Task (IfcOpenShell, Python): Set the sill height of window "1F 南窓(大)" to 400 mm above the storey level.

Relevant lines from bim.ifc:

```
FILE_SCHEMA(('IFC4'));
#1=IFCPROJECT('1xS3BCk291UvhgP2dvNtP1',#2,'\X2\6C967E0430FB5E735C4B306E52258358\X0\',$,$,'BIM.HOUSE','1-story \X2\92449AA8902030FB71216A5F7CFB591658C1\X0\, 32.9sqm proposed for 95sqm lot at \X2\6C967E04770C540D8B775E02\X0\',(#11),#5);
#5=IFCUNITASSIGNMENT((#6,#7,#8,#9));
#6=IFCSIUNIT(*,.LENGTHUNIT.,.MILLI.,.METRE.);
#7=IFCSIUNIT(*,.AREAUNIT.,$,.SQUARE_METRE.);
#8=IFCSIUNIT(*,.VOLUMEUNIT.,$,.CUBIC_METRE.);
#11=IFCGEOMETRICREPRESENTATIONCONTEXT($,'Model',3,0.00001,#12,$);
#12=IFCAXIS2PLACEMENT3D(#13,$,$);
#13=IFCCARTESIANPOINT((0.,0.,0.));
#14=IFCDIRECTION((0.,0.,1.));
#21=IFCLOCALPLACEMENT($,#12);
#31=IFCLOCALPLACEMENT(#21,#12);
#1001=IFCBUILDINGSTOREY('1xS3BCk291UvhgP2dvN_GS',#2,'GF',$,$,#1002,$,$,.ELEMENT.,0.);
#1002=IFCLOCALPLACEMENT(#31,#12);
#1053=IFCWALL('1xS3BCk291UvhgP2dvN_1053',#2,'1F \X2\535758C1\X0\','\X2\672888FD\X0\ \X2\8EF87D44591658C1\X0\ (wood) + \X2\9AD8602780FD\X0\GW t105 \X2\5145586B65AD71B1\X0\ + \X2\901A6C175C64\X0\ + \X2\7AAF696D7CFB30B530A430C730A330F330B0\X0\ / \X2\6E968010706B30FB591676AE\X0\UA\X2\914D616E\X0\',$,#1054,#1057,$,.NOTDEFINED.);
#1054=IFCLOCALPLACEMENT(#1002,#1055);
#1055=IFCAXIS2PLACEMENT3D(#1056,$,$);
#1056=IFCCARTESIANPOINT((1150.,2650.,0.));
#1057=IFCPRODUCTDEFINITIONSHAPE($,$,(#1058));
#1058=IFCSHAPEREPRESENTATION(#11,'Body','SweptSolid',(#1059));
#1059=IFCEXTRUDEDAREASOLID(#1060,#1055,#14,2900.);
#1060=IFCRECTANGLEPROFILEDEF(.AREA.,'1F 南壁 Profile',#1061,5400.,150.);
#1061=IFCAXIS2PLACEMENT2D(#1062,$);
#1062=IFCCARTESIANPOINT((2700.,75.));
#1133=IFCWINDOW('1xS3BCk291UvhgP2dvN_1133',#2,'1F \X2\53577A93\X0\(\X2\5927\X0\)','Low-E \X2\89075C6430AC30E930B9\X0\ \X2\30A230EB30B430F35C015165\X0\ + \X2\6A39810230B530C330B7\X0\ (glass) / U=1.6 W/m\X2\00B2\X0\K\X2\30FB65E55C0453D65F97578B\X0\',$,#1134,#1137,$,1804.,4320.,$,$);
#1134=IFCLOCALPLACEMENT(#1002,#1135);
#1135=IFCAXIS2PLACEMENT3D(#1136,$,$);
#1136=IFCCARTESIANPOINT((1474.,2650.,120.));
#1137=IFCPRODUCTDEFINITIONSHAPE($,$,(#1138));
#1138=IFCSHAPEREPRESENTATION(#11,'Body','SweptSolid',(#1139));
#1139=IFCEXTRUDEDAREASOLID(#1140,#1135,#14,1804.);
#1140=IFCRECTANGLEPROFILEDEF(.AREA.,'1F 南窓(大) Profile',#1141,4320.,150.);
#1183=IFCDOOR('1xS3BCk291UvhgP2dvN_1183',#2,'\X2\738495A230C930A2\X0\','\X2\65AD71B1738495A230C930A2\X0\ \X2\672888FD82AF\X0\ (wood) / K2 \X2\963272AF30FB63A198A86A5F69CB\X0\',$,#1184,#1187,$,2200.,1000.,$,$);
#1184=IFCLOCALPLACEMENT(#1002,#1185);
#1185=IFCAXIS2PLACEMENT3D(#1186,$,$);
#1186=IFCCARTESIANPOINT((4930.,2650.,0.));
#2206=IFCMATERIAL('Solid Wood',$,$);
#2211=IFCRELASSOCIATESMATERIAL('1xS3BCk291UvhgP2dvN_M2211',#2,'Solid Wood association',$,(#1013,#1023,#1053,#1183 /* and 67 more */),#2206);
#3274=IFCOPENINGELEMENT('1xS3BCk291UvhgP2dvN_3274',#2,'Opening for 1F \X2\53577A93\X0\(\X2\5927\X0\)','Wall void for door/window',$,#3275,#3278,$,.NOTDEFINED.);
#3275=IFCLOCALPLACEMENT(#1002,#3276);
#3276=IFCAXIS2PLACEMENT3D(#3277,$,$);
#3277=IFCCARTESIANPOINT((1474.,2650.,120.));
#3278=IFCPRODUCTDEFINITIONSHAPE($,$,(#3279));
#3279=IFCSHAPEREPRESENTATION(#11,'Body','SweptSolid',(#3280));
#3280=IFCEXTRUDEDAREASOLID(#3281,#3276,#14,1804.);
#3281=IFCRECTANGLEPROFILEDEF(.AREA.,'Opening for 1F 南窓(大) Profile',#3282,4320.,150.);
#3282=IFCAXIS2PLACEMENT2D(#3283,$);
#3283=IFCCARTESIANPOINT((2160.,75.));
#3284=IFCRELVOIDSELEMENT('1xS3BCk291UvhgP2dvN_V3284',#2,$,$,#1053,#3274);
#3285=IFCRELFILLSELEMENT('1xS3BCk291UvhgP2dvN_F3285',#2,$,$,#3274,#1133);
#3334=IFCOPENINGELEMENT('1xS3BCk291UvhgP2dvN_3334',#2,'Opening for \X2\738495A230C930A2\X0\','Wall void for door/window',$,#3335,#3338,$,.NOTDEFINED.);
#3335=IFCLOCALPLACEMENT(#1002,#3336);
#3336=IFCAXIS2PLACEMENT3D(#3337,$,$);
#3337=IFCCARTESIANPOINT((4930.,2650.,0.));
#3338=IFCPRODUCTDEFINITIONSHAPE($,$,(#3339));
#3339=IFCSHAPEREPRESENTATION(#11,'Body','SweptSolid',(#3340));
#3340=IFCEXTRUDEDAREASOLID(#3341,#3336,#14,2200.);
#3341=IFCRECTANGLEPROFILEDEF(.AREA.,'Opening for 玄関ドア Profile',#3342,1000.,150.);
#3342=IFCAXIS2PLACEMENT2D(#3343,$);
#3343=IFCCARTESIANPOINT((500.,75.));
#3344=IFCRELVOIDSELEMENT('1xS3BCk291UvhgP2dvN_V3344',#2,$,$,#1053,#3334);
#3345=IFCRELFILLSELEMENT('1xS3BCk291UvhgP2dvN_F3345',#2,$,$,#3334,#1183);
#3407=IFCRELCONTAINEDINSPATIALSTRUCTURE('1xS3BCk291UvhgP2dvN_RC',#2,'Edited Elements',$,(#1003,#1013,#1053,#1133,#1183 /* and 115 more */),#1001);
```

```python
import numpy as np
import ifcopenshell
import ifcopenshell.api.geometry
import ifcopenshell.geom
import ifcopenshell.util.element
import ifcopenshell.util.placement
import ifcopenshell.util.shape
import ifcopenshell.util.unit

model = ifcopenshell.open("bim.ifc")
unit_scale = ifcopenshell.util.unit.calculate_unit_scale(model)

window = model.by_guid("1xS3BCk291UvhgP2dvN_1133")
opening = window.FillsVoids[0].RelatingOpeningElement
storey = ifcopenshell.util.element.get_container(window, ifc_class="IfcBuildingStorey")
level = ifcopenshell.util.placement.get_local_placement(storey.ObjectPlacement)[2, 3]

# The opening's origin need not be at the sill, so measure its lowest point.
shape = ifcopenshell.geom.create_shape(ifcopenshell.geom.settings(), opening)
bottom = ifcopenshell.util.shape.get_shape_bottom_elevation(shape, shape.geometry) / unit_scale
dz = level + 400.0 - bottom

shift = np.array([0.0, 0.0, dz])
# The window is not placed relative to its opening, so move both.
for product in (opening, window):
    matrix = ifcopenshell.util.placement.get_local_placement(product.ObjectPlacement)
    matrix[:3, 3] += shift
    ifcopenshell.api.geometry.edit_object_placement(model, product=product, matrix=matrix, is_si=False)

print(f"moved by {dz * unit_scale:+.3f} m")

model.write("bim_edited.ifc")
```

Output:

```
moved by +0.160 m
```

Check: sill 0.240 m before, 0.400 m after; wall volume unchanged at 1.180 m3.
